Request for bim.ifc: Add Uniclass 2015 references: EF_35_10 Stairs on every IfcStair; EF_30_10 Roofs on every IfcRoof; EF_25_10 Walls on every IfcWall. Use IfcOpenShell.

First a look at what the model holds.

```python
import ifcopenshell

model = ifcopenshell.open("bim.ifc")
print(model.schema)
print("classifications:", [c.Name for c in model.by_type("IfcClassification")])
for ifc_class in ("IfcDoor", "IfcRoof", "IfcStair", "IfcWall", "IfcWindow"):
    print(ifc_class, len(model.by_type(ifc_class)))
```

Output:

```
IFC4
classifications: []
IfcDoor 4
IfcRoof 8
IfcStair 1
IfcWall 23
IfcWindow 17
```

```python
import ifcopenshell
import ifcopenshell.api.classification

model = ifcopenshell.open("bim.ifc")

system = ifcopenshell.api.classification.add_classification(model, classification="Uniclass 2015")

codes = {
    "IfcStair": ("EF_35_10", "Stairs"),
    "IfcRoof": ("EF_30_10", "Roofs"),
    "IfcWall": ("EF_25_10", "Walls"),
}
for ifc_class, (code, name) in codes.items():
    products = model.by_type(ifc_class)
    ifcopenshell.api.classification.add_reference(
        model, products=products, classification=system, identification=code, name=name
    )
    print(code, len(products))

model.write("bim-out.ifc")
```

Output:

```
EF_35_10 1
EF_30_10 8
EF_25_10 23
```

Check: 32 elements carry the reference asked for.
